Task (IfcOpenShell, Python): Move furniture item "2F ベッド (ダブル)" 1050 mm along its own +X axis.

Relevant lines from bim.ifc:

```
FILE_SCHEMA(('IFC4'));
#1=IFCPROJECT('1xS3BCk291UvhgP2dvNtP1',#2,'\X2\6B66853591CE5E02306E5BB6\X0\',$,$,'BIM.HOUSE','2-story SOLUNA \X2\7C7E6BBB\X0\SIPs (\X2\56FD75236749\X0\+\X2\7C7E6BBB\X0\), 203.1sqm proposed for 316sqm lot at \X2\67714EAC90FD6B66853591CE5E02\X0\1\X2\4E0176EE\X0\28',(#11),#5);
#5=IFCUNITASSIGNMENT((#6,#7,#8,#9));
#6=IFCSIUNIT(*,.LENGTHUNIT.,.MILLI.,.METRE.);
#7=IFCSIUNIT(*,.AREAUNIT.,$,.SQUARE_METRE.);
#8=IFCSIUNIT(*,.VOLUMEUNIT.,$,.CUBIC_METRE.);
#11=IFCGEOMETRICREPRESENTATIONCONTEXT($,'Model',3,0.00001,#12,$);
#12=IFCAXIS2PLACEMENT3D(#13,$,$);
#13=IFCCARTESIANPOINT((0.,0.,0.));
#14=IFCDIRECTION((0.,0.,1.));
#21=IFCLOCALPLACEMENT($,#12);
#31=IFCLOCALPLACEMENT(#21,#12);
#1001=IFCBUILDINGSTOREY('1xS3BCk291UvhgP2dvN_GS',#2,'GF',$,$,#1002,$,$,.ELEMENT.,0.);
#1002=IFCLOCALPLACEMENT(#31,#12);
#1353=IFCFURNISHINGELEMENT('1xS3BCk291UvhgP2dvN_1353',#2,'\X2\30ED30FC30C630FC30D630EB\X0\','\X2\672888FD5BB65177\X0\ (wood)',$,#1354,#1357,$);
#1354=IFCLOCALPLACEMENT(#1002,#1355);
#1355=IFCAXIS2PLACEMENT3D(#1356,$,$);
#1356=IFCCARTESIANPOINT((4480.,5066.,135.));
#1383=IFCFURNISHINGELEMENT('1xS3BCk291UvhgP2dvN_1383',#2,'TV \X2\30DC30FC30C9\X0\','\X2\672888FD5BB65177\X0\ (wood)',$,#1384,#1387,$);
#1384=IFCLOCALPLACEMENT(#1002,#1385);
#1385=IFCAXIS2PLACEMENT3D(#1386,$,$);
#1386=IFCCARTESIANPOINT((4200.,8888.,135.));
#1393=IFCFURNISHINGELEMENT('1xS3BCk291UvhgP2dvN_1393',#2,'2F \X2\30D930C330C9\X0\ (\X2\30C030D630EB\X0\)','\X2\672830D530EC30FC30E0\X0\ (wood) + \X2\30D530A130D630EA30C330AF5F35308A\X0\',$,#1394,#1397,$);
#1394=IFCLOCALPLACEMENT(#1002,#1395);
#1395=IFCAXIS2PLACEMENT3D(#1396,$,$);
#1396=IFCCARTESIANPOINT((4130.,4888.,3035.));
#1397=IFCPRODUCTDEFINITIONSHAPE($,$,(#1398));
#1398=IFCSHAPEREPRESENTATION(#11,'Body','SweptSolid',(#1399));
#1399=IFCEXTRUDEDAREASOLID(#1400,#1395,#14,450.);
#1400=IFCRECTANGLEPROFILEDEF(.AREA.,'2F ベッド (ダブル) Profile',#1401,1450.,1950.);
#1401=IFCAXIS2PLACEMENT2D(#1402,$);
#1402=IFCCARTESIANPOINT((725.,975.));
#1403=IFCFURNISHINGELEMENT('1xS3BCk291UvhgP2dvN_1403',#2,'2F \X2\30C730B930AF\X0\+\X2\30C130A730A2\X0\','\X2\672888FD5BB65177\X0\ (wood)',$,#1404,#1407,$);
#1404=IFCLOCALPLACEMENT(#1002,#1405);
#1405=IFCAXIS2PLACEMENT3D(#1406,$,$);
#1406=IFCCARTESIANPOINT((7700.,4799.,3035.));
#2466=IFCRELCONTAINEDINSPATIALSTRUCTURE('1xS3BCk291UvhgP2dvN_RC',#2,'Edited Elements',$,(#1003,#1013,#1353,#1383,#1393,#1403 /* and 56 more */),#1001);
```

```python
import ifcopenshell
import ifcopenshell.api.geometry
import ifcopenshell.util.placement
import ifcopenshell.util.unit

model = ifcopenshell.open("bim.ifc")
unit_scale = ifcopenshell.util.unit.calculate_unit_scale(model)

item = model.by_guid("1xS3BCk291UvhgP2dvN_1393")
matrix = ifcopenshell.util.placement.get_local_placement(item.ObjectPlacement)
matrix[:3, 3] += matrix[:3, 0] * 1.05 / unit_scale
ifcopenshell.api.geometry.edit_object_placement(model, product=item, matrix=matrix, is_si=False)

print(ifcopenshell.util.placement.get_local_placement(item.ObjectPlacement).round(3) + 0.0)

model.write("bim_edited.ifc")
```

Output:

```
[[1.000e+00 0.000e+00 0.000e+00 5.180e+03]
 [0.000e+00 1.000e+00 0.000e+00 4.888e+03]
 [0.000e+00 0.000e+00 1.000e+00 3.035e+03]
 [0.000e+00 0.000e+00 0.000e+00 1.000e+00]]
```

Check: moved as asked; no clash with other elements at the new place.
